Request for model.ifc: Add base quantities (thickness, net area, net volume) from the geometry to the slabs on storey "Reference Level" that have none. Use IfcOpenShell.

First a look at what the model holds.

```python
import ifcopenshell
import ifcopenshell.util.element
import ifcopenshell.util.unit

model = ifcopenshell.open("model.ifc")
print(model.schema)
for unit_type in ("LENGTHUNIT", "AREAUNIT", "VOLUMEUNIT"):
    print(unit_type, ifcopenshell.util.unit.calculate_unit_scale(model, unit_type))
storey = next(s for s in model.by_type("IfcBuildingStorey") if s.Name == "Reference Level")
slabs = [e for e in ifcopenshell.util.element.get_decomposition(storey) if e.is_a("IfcSlab")]
for e in sorted(slabs, key=lambda e: e.id()):
    print(e.id(), e.is_a(), e.Name, list(ifcopenshell.util.element.get_psets(e, qtos_only=True)), sep=" | ")
```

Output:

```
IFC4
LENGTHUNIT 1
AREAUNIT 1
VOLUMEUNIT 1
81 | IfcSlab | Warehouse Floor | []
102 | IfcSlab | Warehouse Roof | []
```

```python
import ifcopenshell
import ifcopenshell.api.pset
import ifcopenshell.geom
import ifcopenshell.util.element
import ifcopenshell.util.shape
import ifcopenshell.util.unit

model = ifcopenshell.open("model.ifc")
unit_scale = ifcopenshell.util.unit.calculate_unit_scale(model)
area_scale = ifcopenshell.util.unit.calculate_unit_scale(model, "AREAUNIT")
volume_scale = ifcopenshell.util.unit.calculate_unit_scale(model, "VOLUMEUNIT")
settings = ifcopenshell.geom.settings()

storey = next(s for s in model.by_type("IfcBuildingStorey") if s.Name == "Reference Level")
slabs = [e for e in ifcopenshell.util.element.get_decomposition(storey) if e.is_a("IfcSlab")]

for e in sorted(slabs, key=lambda e: e.id()):
    if ifcopenshell.util.element.get_psets(e, qtos_only=True, should_inherit=False):
        continue
    # Geometry comes back in metres, in the element's own axes.
    shape = ifcopenshell.geom.create_shape(settings, e)
    values = {
        "Width": ifcopenshell.util.shape.get_z(shape.geometry) / unit_scale,
        "NetArea": ifcopenshell.util.shape.get_footprint_area(shape.geometry) / area_scale,
        "NetVolume": ifcopenshell.util.shape.get_volume(shape.geometry) / volume_scale,
    }
    qto = ifcopenshell.api.pset.add_qto(model, product=e, name="Qto_SlabBaseQuantities")
    ifcopenshell.api.pset.edit_qto(model, qto=qto, properties=values)
    print(e.id(), {k: round(v, 3) for k, v in values.items()})

model.write("model_v2.ifc")
```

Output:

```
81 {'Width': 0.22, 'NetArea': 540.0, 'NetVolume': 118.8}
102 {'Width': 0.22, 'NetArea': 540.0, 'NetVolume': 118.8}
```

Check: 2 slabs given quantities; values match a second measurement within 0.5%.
